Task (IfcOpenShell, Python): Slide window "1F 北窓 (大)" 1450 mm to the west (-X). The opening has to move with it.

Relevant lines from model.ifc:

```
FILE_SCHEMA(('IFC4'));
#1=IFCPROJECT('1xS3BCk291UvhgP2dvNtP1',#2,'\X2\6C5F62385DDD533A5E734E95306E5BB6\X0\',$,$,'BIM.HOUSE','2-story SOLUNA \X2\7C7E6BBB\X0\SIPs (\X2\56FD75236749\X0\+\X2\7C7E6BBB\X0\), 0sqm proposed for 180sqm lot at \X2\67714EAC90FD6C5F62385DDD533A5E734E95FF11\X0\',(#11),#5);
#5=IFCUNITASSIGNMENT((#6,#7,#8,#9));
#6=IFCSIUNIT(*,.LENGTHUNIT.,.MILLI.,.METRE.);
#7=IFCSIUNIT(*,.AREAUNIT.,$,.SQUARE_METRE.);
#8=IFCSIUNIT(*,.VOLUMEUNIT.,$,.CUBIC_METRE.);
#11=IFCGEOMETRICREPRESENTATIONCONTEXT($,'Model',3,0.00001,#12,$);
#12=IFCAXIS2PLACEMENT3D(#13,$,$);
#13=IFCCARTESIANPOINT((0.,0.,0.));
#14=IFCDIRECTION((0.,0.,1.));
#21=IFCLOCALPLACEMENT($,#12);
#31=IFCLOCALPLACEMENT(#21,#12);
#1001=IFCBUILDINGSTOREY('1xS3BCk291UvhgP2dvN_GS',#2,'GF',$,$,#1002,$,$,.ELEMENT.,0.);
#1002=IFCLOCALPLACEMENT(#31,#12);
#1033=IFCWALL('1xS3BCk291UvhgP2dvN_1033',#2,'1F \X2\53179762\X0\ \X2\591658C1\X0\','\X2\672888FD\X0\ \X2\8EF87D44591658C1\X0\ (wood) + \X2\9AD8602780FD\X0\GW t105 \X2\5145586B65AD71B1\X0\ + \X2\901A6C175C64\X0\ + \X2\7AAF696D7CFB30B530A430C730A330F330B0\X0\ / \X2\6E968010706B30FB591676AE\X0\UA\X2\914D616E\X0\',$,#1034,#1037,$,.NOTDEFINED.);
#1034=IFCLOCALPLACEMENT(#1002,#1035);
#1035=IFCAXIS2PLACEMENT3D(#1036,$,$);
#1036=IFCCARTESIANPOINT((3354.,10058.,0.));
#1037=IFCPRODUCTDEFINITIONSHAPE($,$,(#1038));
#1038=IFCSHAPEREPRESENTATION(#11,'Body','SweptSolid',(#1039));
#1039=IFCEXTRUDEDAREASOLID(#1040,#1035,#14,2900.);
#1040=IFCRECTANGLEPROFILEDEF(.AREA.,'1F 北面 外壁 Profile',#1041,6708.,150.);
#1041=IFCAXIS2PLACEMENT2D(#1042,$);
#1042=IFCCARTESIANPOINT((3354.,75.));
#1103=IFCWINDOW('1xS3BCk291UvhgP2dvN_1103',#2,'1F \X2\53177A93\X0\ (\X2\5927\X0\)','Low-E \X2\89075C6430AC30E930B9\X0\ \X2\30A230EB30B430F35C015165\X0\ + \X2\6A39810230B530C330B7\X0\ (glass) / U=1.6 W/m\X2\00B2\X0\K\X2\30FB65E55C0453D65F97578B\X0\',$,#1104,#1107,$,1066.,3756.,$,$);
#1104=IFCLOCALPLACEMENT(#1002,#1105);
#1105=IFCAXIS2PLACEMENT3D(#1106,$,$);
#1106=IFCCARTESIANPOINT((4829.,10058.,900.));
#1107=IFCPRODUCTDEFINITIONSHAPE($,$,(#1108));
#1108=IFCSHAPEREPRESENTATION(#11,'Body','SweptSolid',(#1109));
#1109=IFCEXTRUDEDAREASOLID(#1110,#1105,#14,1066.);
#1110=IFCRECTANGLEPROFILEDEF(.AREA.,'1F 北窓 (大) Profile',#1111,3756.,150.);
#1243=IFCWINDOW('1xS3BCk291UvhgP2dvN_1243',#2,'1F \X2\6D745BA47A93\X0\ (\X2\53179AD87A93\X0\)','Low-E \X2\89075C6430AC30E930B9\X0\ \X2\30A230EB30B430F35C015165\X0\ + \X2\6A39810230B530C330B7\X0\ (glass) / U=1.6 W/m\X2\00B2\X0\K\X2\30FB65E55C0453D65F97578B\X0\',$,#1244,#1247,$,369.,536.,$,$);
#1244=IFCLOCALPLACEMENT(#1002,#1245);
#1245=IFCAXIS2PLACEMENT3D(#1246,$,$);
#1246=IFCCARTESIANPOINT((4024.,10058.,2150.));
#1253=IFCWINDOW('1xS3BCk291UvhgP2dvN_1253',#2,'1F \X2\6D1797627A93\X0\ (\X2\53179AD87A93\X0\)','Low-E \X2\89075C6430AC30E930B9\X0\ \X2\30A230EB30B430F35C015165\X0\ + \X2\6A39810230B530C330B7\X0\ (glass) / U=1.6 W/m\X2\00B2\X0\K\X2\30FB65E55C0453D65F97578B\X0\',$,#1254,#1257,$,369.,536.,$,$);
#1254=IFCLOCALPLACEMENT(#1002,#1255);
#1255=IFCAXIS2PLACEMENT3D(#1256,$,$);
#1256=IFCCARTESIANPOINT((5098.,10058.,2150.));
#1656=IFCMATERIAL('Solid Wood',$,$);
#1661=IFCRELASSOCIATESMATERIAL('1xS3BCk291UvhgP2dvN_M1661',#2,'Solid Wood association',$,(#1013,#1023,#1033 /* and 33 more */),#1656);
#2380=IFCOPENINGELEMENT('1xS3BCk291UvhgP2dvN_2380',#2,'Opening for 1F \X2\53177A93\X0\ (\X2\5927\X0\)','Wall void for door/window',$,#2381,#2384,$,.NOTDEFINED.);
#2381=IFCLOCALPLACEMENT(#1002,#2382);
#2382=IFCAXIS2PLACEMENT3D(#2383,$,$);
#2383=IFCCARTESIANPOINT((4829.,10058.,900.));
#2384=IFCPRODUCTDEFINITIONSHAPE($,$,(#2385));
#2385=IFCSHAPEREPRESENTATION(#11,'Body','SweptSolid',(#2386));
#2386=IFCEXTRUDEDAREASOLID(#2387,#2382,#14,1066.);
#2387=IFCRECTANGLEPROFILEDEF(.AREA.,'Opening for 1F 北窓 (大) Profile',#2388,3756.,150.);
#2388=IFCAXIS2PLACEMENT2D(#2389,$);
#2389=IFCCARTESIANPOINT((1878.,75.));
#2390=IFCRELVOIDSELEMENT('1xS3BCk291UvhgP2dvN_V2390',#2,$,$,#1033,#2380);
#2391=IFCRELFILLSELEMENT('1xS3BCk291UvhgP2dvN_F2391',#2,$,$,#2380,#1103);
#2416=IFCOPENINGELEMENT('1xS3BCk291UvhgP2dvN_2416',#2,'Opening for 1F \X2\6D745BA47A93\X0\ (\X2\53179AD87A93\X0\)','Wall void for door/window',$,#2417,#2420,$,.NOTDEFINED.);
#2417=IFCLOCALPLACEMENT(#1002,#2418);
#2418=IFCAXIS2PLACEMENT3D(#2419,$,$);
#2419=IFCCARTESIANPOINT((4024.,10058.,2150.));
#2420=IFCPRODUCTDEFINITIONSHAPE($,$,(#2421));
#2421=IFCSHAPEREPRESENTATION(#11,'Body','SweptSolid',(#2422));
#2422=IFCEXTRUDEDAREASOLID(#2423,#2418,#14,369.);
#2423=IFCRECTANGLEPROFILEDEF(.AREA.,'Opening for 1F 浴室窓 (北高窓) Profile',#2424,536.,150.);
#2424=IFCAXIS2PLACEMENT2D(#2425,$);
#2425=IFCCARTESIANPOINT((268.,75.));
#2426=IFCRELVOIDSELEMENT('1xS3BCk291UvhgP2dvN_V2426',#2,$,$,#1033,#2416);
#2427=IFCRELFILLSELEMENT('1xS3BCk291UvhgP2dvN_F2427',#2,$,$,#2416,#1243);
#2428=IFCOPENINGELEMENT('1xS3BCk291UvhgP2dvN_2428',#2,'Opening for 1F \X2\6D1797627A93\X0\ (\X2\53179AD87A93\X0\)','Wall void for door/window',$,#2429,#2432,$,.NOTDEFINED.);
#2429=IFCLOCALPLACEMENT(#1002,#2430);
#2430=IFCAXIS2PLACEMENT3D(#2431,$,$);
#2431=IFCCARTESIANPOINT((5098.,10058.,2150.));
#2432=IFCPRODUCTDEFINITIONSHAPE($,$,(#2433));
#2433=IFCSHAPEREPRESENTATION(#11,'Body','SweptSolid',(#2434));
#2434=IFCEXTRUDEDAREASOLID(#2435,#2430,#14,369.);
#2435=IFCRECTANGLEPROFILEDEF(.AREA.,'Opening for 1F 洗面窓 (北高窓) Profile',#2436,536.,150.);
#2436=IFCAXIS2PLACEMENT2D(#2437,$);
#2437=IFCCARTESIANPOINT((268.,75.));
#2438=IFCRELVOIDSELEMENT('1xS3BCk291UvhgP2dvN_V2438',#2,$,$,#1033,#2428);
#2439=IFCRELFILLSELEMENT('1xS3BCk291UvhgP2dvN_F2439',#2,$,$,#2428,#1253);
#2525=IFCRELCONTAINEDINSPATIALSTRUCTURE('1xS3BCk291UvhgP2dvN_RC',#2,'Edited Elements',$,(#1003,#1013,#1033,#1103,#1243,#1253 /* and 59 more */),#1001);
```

```python
import ifcopenshell
import ifcopenshell.api.geometry
import ifcopenshell.util.placement
import ifcopenshell.util.unit

model = ifcopenshell.open("model.ifc")
unit_scale = ifcopenshell.util.unit.calculate_unit_scale(model)

window = model.by_guid("1xS3BCk291UvhgP2dvN_1103")
opening = window.FillsVoids[0].RelatingOpeningElement
wall = opening.VoidsElements[0].RelatingBuildingElement

wall_matrix = ifcopenshell.util.placement.get_local_placement(wall.ObjectPlacement)
shift = wall_matrix[:3, 0] * -1.45 / unit_scale
before = ifcopenshell.util.placement.get_local_placement(window.ObjectPlacement)[:3, 3].copy()

# The window is not placed relative to its opening, so move both.
for product in (opening, window):
    matrix = ifcopenshell.util.placement.get_local_placement(product.ObjectPlacement)
    matrix[:3, 3] += shift
    ifcopenshell.api.geometry.edit_object_placement(model, product=product, matrix=matrix, is_si=False)

after = ifcopenshell.util.placement.get_local_placement(window.ObjectPlacement)[:3, 3]
print("window moved by", (after - before).round(3) + 0.0)

model.write("model_v2.ifc")
```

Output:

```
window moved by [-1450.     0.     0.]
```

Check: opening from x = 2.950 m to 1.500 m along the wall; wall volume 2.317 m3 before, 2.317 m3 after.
